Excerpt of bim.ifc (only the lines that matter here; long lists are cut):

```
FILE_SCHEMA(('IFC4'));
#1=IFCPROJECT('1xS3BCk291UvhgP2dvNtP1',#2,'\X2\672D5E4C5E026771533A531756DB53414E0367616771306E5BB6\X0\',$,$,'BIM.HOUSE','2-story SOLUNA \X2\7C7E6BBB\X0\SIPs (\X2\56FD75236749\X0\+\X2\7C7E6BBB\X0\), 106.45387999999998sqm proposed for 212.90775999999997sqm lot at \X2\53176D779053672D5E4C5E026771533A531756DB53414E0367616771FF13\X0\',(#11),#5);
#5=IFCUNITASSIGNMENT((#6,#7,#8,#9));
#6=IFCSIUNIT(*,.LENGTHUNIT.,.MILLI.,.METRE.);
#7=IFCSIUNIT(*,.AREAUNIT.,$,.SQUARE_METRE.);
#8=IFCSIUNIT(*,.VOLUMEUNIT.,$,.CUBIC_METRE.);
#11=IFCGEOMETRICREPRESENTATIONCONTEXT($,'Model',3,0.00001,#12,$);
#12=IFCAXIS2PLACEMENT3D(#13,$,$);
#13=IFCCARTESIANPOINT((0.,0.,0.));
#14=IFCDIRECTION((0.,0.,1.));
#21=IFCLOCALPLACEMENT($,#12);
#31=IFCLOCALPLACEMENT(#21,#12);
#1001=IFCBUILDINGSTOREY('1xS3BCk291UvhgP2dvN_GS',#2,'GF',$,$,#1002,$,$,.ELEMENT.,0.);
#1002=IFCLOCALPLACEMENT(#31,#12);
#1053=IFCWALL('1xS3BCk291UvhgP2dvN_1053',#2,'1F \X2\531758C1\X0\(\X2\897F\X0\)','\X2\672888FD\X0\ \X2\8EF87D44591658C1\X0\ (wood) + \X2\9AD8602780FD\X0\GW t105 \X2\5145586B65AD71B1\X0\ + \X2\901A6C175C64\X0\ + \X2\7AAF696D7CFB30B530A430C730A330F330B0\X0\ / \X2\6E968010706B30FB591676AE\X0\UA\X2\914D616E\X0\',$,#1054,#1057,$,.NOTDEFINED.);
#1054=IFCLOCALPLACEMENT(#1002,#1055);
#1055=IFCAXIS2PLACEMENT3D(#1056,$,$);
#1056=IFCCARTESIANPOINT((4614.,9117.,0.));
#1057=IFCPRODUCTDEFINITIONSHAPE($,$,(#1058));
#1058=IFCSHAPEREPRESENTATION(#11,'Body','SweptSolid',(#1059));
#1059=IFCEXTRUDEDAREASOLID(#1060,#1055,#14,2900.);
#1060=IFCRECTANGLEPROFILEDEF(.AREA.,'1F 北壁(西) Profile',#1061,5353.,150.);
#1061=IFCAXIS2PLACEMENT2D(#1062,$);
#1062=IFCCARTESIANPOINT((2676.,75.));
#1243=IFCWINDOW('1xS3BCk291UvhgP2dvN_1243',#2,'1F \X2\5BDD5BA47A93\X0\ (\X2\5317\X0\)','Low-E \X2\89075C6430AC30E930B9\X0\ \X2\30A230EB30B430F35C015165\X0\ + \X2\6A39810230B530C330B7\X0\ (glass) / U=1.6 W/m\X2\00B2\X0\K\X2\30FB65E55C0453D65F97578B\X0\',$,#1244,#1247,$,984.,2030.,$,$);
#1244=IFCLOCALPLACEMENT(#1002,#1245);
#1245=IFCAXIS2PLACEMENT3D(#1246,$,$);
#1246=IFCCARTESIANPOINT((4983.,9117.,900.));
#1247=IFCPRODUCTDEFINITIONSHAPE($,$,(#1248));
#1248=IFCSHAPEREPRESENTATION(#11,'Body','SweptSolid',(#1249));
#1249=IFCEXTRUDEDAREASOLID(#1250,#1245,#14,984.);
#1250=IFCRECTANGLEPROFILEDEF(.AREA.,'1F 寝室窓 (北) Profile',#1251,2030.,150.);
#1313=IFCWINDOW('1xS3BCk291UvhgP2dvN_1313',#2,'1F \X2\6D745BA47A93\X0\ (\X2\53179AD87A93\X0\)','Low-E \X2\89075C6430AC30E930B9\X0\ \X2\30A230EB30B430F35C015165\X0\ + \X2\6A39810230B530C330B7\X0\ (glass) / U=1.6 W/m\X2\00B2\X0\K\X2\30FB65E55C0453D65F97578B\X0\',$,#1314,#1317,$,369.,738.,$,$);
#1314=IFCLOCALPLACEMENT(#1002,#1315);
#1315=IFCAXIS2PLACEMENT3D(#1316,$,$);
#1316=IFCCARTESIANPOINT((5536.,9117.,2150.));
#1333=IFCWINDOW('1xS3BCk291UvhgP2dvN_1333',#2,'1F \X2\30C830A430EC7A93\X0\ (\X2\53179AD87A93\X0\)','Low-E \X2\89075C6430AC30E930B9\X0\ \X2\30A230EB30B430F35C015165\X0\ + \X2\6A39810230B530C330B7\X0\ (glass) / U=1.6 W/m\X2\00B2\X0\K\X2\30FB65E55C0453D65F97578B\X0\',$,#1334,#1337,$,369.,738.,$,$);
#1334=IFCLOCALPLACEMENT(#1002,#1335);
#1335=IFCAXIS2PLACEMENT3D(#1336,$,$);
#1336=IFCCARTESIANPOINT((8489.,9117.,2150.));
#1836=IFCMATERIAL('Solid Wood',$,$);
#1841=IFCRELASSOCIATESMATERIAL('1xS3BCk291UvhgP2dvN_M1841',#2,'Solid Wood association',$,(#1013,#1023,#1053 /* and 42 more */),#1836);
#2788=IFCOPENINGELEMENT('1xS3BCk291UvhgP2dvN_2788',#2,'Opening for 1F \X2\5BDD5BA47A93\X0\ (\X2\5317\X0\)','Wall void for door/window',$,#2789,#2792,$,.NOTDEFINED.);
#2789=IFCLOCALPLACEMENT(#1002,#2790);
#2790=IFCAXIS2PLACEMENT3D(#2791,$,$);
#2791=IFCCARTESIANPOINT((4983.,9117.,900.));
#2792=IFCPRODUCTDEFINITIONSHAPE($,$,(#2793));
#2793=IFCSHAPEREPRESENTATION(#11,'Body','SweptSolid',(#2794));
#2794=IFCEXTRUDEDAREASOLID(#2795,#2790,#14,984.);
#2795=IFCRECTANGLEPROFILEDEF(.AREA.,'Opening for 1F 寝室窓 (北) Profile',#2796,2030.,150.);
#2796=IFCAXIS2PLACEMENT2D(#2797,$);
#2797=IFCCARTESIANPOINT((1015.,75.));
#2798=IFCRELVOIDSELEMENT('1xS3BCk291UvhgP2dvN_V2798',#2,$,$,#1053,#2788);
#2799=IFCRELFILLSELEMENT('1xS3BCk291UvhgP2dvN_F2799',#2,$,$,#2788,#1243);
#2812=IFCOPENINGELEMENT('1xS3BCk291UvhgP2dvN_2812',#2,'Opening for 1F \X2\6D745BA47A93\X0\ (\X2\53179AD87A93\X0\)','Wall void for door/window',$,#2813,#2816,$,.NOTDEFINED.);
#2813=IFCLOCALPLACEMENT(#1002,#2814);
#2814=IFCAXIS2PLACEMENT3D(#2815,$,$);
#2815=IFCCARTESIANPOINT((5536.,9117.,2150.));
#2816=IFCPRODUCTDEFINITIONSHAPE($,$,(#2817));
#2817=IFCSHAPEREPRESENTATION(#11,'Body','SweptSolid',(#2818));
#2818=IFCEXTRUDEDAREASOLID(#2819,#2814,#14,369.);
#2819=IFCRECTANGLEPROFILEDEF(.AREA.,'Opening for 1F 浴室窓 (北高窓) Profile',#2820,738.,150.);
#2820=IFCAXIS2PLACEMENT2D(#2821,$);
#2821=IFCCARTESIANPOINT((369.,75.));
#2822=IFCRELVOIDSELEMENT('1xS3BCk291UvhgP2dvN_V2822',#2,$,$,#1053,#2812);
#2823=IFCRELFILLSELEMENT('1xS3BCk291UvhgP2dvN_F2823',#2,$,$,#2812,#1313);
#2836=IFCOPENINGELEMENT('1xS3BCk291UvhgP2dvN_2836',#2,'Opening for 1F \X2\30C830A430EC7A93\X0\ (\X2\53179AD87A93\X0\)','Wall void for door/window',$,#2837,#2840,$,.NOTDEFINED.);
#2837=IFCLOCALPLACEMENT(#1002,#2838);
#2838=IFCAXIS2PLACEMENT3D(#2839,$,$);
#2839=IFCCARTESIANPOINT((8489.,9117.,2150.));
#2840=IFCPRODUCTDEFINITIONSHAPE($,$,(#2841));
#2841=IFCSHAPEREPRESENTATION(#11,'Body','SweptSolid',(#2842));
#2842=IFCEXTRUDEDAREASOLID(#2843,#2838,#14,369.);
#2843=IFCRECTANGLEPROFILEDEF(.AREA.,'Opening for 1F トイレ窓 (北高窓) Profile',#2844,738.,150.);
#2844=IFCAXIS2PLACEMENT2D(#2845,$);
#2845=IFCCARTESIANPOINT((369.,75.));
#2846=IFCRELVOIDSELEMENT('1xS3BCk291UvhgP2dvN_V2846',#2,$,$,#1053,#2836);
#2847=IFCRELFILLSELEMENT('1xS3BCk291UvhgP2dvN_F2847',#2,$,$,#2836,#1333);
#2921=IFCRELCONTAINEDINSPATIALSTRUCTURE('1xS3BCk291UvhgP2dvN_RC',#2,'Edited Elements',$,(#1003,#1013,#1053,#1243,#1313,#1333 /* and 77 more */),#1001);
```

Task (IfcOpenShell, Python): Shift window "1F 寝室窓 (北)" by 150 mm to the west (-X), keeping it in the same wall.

```python
import ifcopenshell
import ifcopenshell.api.geometry
import ifcopenshell.util.placement
import ifcopenshell.util.unit

model = ifcopenshell.open("bim.ifc")
unit_scale = ifcopenshell.util.unit.calculate_unit_scale(model)

window = model.by_guid("1xS3BCk291UvhgP2dvN_1243")
opening = window.FillsVoids[0].RelatingOpeningElement
wall = opening.VoidsElements[0].RelatingBuildingElement

wall_matrix = ifcopenshell.util.placement.get_local_placement(wall.ObjectPlacement)
shift = wall_matrix[:3, 0] * -0.15 / unit_scale
before = ifcopenshell.util.placement.get_local_placement(window.ObjectPlacement)[:3, 3].copy()

# The window is not placed relative to its opening, so move both.
for product in (opening, window):
    matrix = ifcopenshell.util.placement.get_local_placement(product.ObjectPlacement)
    matrix[:3, 3] += shift
    ifcopenshell.api.geometry.edit_object_placement(model, product=product, matrix=matrix, is_si=False)

after = ifcopenshell.util.placement.get_local_placement(window.ObjectPlacement)[:3, 3]
print("window moved by", (after - before).round(3) + 0.0)

model.write("bim-out.ifc")
```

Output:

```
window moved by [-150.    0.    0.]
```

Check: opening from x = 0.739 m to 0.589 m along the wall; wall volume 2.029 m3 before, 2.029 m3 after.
